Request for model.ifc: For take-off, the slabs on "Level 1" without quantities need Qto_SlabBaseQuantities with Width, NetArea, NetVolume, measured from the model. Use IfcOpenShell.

First a look at what the model holds.

```python
import ifcopenshell
import ifcopenshell.util.element
import ifcopenshell.util.unit

model = ifcopenshell.open("model.ifc")
print(model.schema)
for unit_type in ("LENGTHUNIT", "AREAUNIT", "VOLUMEUNIT"):
    print(unit_type, ifcopenshell.util.unit.calculate_unit_scale(model, unit_type))
storey = next(s for s in model.by_type("IfcBuildingStorey") if s.Name == "Level 1")
slabs = [e for e in ifcopenshell.util.element.get_decomposition(storey) if e.is_a("IfcSlab")]
for e in sorted(slabs, key=lambda e: e.id()):
    print(e.id(), e.is_a(), e.Name, list(ifcopenshell.util.element.get_psets(e, qtos_only=True)), sep=" | ")
```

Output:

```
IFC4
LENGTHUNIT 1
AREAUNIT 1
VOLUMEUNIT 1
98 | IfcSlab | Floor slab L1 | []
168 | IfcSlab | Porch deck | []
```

```python
import ifcopenshell
import ifcopenshell.api.pset
import ifcopenshell.geom
import ifcopenshell.util.element
import ifcopenshell.util.shape
import ifcopenshell.util.unit

model = ifcopenshell.open("model.ifc")
unit_scale = ifcopenshell.util.unit.calculate_unit_scale(model)
area_scale = ifcopenshell.util.unit.calculate_unit_scale(model, "AREAUNIT")
volume_scale = ifcopenshell.util.unit.calculate_unit_scale(model, "VOLUMEUNIT")
settings = ifcopenshell.geom.settings()

storey = next(s for s in model.by_type("IfcBuildingStorey") if s.Name == "Level 1")
slabs = [e for e in ifcopenshell.util.element.get_decomposition(storey) if e.is_a("IfcSlab")]

for e in sorted(slabs, key=lambda e: e.id()):
    if ifcopenshell.util.element.get_psets(e, qtos_only=True, should_inherit=False):
        continue
    # Geometry comes back in metres, in the element's own axes.
    shape = ifcopenshell.geom.create_shape(settings, e)
    values = {
        "Width": ifcopenshell.util.shape.get_z(shape.geometry) / unit_scale,
        "NetArea": ifcopenshell.util.shape.get_footprint_area(shape.geometry) / area_scale,
        "NetVolume": ifcopenshell.util.shape.get_volume(shape.geometry) / volume_scale,
    }
    qto = ifcopenshell.api.pset.add_qto(model, product=e, name="Qto_SlabBaseQuantities")
    ifcopenshell.api.pset.edit_qto(model, qto=qto, properties=values)
    print(e.id(), {k: round(v, 3) for k, v in values.items()})

model.write("model_v2.ifc")
```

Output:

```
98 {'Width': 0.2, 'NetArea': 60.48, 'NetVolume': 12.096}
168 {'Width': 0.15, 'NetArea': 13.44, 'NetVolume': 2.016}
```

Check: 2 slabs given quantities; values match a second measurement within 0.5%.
